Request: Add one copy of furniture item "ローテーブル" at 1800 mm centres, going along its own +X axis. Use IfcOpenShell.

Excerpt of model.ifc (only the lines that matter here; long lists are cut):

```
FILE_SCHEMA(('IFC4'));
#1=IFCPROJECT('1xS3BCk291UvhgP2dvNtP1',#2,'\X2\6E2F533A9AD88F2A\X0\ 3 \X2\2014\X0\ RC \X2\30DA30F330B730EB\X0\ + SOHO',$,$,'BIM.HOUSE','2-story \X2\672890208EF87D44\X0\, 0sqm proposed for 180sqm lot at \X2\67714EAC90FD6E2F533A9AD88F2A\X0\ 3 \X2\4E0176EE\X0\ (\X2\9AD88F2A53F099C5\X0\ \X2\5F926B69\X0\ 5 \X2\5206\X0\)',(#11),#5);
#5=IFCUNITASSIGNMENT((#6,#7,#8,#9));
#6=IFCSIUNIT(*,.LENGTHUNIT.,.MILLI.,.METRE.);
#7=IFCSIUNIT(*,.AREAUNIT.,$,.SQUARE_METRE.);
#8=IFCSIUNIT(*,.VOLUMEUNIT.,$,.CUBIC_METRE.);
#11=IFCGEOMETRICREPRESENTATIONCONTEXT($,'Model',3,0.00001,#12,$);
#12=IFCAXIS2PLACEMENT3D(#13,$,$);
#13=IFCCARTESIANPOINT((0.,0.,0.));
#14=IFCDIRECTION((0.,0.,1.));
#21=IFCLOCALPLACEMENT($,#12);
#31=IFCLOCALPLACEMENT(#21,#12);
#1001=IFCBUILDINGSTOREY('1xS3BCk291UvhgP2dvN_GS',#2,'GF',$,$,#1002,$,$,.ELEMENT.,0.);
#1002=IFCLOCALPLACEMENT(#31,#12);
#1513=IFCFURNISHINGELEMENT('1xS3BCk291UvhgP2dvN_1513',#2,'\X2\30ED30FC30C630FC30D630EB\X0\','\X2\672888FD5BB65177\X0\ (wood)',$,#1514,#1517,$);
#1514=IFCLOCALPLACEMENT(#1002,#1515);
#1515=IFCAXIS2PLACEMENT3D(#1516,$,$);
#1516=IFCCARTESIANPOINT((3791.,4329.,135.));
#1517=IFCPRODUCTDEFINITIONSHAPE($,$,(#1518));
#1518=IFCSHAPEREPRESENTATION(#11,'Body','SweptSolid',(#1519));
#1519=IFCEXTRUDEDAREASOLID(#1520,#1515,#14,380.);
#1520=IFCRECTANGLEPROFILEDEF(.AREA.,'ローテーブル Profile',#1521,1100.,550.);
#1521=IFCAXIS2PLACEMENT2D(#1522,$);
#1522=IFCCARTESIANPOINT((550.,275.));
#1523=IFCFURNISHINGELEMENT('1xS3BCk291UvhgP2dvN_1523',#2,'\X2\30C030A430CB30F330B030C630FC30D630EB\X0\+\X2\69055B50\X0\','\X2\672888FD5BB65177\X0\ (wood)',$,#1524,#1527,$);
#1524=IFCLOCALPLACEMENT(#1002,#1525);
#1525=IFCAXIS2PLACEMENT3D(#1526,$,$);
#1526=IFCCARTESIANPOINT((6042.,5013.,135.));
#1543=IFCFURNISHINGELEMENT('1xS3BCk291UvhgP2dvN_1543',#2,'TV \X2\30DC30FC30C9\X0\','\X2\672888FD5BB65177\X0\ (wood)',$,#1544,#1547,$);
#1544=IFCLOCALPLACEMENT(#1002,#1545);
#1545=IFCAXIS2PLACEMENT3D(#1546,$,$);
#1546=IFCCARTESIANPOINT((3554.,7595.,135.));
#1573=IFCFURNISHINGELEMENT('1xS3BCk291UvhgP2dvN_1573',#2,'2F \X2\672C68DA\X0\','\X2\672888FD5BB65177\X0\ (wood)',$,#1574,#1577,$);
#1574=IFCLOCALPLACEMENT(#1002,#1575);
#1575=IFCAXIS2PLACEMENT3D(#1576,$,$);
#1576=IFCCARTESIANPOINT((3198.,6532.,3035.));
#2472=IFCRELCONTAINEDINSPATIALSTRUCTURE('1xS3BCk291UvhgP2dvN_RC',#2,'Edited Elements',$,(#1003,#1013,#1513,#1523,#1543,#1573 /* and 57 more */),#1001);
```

```python
import ifcopenshell
import ifcopenshell.api.geometry
import ifcopenshell.api.root
import ifcopenshell.util.element
import ifcopenshell.util.placement
import ifcopenshell.util.unit

model = ifcopenshell.open("model.ifc")
unit_scale = ifcopenshell.util.unit.calculate_unit_scale(model)


def reuse_history(source, copy):
    """copy_class also copies each property set's owner history, people and application; keep the originals."""
    for rel in copy.IsDefinedBy:
        if rel.is_a("IfcRelDefinesByProperties") and (history := rel.RelatingPropertyDefinition.OwnerHistory):
            rel.RelatingPropertyDefinition.OwnerHistory = source.OwnerHistory
            ifcopenshell.util.element.remove_deep2(model, history)


source = model.by_guid("1xS3BCk291UvhgP2dvN_1513")
base = ifcopenshell.util.placement.get_local_placement(source.ObjectPlacement)
step = base[:3, 0] * 1.8 / unit_scale

for i in range(1, 2):
    copy = ifcopenshell.api.root.copy_class(model, product=source)
    copy.Representation = ifcopenshell.util.element.copy_deep(
        model, source.Representation, exclude=["IfcGeometricRepresentationContext", "IfcRepresentationMap"]
    )
    reuse_history(source, copy)
    matrix = base.copy()
    matrix[:3, 3] += i * step
    print("added at", matrix[:3, 3].round(3) + 0.0)
    ifcopenshell.api.geometry.edit_object_placement(model, product=copy, matrix=matrix, is_si=False)

model.write("model-out.ifc")
```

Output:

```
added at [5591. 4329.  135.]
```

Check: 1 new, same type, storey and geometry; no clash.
